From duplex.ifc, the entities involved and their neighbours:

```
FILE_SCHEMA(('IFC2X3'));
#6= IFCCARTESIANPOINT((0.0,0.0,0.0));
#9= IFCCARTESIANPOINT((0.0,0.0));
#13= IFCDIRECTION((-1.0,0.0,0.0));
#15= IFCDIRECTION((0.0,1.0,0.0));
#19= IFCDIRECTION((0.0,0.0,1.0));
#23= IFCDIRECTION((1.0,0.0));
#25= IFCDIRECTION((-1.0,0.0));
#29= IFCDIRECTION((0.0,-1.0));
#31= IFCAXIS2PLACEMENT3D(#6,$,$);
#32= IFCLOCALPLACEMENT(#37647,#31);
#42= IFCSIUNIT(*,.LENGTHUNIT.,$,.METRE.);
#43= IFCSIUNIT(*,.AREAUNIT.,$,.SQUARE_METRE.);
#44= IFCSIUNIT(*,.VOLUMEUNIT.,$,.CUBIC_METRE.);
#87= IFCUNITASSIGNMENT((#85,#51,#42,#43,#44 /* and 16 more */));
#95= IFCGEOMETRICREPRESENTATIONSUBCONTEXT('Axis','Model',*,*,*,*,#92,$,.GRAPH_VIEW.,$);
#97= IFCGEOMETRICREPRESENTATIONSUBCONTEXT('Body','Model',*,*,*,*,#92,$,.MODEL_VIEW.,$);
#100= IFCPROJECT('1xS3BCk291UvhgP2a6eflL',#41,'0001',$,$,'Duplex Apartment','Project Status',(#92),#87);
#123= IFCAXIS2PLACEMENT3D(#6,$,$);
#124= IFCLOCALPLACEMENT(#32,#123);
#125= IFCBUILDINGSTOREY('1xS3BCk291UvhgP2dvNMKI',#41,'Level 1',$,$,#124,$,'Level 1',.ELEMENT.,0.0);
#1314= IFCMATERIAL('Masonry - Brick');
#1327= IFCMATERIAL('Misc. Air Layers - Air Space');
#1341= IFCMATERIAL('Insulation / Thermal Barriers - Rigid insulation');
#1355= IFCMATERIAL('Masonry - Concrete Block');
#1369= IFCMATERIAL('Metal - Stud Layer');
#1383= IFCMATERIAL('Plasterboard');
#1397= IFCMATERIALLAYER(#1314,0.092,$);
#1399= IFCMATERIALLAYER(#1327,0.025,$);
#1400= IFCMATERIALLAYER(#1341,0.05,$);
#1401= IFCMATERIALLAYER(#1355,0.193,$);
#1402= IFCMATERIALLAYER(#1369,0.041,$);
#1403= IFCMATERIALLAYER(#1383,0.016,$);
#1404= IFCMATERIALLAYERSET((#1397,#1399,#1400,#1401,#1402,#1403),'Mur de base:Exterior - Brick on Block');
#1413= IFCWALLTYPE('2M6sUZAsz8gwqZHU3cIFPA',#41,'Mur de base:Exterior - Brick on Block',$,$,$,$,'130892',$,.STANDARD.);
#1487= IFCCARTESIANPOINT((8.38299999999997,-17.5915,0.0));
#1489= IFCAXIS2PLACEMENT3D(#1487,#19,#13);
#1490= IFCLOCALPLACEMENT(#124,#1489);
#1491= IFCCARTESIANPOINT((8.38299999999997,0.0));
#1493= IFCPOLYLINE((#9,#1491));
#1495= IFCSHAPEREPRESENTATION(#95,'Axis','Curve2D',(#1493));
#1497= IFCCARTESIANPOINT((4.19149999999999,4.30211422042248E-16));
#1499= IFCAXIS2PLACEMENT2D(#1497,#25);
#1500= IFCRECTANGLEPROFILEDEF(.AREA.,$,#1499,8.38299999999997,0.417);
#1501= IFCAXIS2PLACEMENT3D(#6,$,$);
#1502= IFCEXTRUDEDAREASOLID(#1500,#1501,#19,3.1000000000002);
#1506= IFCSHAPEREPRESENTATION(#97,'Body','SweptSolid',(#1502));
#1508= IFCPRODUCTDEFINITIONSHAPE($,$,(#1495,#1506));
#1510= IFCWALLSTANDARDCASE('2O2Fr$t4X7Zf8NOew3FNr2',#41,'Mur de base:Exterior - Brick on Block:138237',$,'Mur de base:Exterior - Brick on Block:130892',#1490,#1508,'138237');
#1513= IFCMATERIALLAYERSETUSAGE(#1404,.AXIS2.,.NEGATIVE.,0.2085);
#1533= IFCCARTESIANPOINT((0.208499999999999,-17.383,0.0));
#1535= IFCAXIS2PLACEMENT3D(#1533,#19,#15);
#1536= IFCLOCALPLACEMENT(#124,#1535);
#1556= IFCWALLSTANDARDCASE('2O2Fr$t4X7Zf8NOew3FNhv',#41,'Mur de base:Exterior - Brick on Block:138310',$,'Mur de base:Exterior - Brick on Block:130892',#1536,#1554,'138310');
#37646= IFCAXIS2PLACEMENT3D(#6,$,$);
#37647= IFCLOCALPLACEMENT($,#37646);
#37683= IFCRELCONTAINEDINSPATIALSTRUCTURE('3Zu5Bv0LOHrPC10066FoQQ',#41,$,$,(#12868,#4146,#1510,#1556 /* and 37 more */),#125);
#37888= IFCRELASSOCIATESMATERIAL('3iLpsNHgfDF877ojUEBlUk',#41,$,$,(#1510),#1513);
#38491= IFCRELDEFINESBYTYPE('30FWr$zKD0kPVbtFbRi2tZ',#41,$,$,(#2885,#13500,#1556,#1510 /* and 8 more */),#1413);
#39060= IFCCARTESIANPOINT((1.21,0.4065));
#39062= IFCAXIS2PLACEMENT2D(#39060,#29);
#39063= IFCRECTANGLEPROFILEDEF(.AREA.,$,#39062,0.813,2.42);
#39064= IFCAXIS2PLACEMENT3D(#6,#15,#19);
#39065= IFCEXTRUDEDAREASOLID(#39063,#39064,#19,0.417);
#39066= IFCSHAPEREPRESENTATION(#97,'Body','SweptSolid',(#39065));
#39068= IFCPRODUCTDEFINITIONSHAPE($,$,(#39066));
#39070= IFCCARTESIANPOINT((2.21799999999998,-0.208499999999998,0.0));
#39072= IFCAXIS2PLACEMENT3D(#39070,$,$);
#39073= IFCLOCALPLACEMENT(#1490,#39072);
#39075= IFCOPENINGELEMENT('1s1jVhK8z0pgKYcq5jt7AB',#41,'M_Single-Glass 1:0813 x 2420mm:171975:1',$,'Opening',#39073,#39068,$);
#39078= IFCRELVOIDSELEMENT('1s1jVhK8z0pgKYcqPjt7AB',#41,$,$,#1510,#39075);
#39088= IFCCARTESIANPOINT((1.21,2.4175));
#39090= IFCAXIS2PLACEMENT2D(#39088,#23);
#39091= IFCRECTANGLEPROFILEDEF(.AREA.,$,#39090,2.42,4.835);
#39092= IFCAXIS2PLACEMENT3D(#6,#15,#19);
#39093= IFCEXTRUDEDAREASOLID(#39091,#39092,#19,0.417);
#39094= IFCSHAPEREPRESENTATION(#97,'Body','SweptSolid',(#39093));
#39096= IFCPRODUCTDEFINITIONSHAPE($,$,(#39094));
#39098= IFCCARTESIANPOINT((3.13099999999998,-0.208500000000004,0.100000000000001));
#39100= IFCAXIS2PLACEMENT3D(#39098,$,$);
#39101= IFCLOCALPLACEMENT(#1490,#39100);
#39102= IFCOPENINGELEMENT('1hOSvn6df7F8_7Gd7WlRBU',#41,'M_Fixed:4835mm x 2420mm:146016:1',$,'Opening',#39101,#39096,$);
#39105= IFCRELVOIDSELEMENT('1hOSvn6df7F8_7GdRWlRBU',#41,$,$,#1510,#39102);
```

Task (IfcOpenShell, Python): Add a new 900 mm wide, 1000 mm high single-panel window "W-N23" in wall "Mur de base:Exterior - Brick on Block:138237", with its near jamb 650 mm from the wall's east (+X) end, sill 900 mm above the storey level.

```python
import numpy as np
import ifcopenshell
import ifcopenshell.api.feature
import ifcopenshell.api.geometry
import ifcopenshell.api.root
import ifcopenshell.api.spatial
import ifcopenshell.api.type
import ifcopenshell.geom
import ifcopenshell.util.element
import ifcopenshell.util.placement
import ifcopenshell.util.representation
import ifcopenshell.util.shape
import ifcopenshell.util.unit

model = ifcopenshell.open("duplex.ifc")
unit_scale = ifcopenshell.util.unit.calculate_unit_scale(model)
settings = ifcopenshell.geom.settings()


def volume(element):
    """Net volume in cubic metres, openings subtracted."""
    shape = ifcopenshell.geom.create_shape(settings, element)
    return ifcopenshell.util.shape.get_volume(shape.geometry)


wall = model.by_guid("2O2Fr$t4X7Zf8NOew3FNr2")
storey = ifcopenshell.util.element.get_container(wall, ifc_class="IfcBuildingStorey")
context = ifcopenshell.util.representation.get_context(model, "Model", "Body", "MODEL_VIEW")
before = volume(wall)

width, height, from_end, sill = 0.9, 1, 0.65, 0.9  # metres

# The wall runs along its own X axis, and the end named is its -X end.
wall_shape = ifcopenshell.geom.create_shape(settings, wall)
x, y, z = ifcopenshell.util.shape.get_vertices(wall_shape.geometry).T
start = x.min() + from_end
face, thickness = float(y.min()), float(y.max() - y.min())
wall_matrix = ifcopenshell.util.placement.get_local_placement(wall.ObjectPlacement)
level = ifcopenshell.util.placement.get_local_placement(storey.ObjectPlacement)[2, 3]


def in_wall(x, y):
    """Placement at x, y metres in the wall's axes, at sill height."""
    matrix = wall_matrix.copy()
    matrix[:, 3] = wall_matrix @ np.array([x / unit_scale, y / unit_scale, 0.0, 1.0])
    matrix[2, 3] = level + sill / unit_scale
    return matrix


# Opening: a box that overshoots both wall faces by 50 mm.
opening = ifcopenshell.api.root.create_entity(model, ifc_class="IfcOpeningElement")
box = ifcopenshell.api.geometry.add_wall_representation(
    model, context=context, length=width, height=height, thickness=thickness + 0.1
)
ifcopenshell.api.geometry.assign_representation(model, product=opening, representation=box)
ifcopenshell.api.geometry.edit_object_placement(model, product=opening, matrix=in_wall(start, face - 0.05), is_si=False)
ifcopenshell.api.feature.add_feature(model, feature=opening, element=wall)

window = ifcopenshell.api.root.create_entity(model, ifc_class="IfcWindow", name="W-N23")
window.OverallWidth, window.OverallHeight = width / unit_scale, height / unit_scale
body = ifcopenshell.api.geometry.add_window_representation(
    model,
    context=context,
    overall_width=window.OverallWidth,
    overall_height=window.OverallHeight,
    partition_type="SINGLE_PANEL",
)
ifcopenshell.api.geometry.assign_representation(model, product=window, representation=body)
ifcopenshell.api.spatial.assign_container(model, products=[window], relating_structure=storey)
fills = ifcopenshell.api.feature.add_filling(model, opening=opening, element=window)
fills.OwnerHistory = window.OwnerHistory  # required in IFC2X3

# IFC2X3 keeps the operation on the window style.
style = ifcopenshell.api.root.create_entity(model, ifc_class="IfcWindowStyle", name="W-N23")
style.OperationType, style.ConstructionType = "SINGLE_PANEL", "NOTDEFINED"
style.ParameterTakesPrecedence = style.Sizeable = False
ifcopenshell.api.type.assign_type(model, related_objects=[window], relating_type=style)

# Centre the window in the wall's thickness.
ifcopenshell.api.geometry.edit_object_placement(model, product=window, matrix=in_wall(start, face), is_si=False)
window_shape = ifcopenshell.geom.create_shape(settings, window)
depth = ifcopenshell.util.shape.get_vertices(window_shape.geometry)[:, 1]
offset = face + thickness / 2 - (depth.min() + depth.max()) / 2
ifcopenshell.api.geometry.edit_object_placement(model, product=window, matrix=in_wall(start, offset), is_si=False)

after = volume(wall)

print(f"wall volume {before:.3f} -> {after:.3f} m3")

model.write("duplex_updated.ifc")
```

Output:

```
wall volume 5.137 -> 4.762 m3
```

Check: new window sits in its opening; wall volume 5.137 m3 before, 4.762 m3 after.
